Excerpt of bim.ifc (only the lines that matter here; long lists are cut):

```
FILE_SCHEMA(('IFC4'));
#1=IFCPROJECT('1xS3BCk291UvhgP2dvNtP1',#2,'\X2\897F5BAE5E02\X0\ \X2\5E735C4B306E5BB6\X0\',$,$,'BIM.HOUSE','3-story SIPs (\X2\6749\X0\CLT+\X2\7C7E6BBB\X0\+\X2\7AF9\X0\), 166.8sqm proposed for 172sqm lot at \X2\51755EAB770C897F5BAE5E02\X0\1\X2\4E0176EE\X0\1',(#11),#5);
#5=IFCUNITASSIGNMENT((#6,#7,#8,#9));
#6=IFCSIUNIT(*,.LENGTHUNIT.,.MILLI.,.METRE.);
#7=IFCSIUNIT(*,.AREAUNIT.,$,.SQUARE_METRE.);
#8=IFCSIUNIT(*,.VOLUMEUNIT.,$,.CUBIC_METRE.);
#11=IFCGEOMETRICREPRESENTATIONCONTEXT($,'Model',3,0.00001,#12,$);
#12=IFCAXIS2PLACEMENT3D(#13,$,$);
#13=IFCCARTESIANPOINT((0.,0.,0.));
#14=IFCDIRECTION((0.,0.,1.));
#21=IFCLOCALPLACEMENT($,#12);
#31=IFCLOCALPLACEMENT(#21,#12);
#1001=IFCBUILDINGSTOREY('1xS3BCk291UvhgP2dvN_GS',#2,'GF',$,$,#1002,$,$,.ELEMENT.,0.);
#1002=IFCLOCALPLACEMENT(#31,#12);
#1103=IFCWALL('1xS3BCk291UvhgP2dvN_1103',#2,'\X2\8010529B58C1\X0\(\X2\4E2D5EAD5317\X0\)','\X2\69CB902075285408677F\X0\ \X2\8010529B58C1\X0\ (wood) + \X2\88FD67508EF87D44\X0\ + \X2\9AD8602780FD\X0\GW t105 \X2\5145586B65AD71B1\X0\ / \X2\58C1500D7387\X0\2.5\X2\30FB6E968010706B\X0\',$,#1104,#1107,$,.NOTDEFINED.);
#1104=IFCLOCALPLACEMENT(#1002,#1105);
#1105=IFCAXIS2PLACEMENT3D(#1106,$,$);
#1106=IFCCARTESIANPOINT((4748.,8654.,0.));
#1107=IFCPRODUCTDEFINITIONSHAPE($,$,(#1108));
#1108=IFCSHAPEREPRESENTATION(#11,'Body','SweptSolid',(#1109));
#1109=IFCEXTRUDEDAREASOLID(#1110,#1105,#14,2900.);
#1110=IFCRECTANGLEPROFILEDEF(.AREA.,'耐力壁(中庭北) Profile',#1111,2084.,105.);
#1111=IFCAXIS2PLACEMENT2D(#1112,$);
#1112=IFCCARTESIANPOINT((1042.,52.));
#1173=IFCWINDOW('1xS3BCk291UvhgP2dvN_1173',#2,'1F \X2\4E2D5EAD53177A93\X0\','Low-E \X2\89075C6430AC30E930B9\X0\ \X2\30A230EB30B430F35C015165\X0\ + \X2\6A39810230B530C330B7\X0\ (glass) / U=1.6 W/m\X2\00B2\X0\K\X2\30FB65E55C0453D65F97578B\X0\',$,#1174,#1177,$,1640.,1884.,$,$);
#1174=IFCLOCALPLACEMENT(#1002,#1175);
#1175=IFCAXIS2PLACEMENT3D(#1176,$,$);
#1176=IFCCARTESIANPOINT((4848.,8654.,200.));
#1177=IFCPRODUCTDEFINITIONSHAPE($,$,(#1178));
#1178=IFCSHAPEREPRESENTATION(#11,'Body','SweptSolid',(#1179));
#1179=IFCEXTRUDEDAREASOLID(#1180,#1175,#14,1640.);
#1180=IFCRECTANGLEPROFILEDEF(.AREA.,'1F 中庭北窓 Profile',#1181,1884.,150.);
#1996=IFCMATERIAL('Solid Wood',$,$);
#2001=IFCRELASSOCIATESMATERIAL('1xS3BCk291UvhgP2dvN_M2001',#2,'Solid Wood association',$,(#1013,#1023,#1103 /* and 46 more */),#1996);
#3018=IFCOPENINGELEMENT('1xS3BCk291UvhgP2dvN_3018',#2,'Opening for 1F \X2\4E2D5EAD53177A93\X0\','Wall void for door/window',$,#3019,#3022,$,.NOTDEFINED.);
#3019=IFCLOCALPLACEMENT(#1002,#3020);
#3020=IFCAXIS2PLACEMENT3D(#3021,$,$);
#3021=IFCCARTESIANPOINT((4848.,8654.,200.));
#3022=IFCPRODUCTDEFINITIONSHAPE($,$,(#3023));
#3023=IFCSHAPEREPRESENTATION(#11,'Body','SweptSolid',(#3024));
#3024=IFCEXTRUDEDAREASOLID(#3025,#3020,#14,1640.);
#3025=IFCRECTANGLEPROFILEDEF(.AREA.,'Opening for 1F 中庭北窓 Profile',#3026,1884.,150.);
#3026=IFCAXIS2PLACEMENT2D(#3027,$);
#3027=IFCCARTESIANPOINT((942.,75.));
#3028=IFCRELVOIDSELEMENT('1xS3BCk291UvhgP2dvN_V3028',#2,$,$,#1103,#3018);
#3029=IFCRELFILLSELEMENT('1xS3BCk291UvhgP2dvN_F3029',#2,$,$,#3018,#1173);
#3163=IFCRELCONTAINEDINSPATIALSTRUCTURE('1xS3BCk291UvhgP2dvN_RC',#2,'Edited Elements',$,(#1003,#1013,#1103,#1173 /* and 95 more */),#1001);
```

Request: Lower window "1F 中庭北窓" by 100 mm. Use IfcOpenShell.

```python
import numpy as np
import ifcopenshell
import ifcopenshell.api.geometry
import ifcopenshell.util.placement
import ifcopenshell.util.unit

model = ifcopenshell.open("bim.ifc")
unit_scale = ifcopenshell.util.unit.calculate_unit_scale(model)

window = model.by_guid("1xS3BCk291UvhgP2dvN_1173")
opening = window.FillsVoids[0].RelatingOpeningElement
dz = -100.0

shift = np.array([0.0, 0.0, dz])
# The window is not placed relative to its opening, so move both.
for product in (opening, window):
    matrix = ifcopenshell.util.placement.get_local_placement(product.ObjectPlacement)
    matrix[:3, 3] += shift
    ifcopenshell.api.geometry.edit_object_placement(model, product=product, matrix=matrix, is_si=False)

print(f"moved by {dz * unit_scale:+.3f} m")

model.write("bim_edited.ifc")
```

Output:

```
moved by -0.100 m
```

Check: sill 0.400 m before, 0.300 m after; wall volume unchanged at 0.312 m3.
